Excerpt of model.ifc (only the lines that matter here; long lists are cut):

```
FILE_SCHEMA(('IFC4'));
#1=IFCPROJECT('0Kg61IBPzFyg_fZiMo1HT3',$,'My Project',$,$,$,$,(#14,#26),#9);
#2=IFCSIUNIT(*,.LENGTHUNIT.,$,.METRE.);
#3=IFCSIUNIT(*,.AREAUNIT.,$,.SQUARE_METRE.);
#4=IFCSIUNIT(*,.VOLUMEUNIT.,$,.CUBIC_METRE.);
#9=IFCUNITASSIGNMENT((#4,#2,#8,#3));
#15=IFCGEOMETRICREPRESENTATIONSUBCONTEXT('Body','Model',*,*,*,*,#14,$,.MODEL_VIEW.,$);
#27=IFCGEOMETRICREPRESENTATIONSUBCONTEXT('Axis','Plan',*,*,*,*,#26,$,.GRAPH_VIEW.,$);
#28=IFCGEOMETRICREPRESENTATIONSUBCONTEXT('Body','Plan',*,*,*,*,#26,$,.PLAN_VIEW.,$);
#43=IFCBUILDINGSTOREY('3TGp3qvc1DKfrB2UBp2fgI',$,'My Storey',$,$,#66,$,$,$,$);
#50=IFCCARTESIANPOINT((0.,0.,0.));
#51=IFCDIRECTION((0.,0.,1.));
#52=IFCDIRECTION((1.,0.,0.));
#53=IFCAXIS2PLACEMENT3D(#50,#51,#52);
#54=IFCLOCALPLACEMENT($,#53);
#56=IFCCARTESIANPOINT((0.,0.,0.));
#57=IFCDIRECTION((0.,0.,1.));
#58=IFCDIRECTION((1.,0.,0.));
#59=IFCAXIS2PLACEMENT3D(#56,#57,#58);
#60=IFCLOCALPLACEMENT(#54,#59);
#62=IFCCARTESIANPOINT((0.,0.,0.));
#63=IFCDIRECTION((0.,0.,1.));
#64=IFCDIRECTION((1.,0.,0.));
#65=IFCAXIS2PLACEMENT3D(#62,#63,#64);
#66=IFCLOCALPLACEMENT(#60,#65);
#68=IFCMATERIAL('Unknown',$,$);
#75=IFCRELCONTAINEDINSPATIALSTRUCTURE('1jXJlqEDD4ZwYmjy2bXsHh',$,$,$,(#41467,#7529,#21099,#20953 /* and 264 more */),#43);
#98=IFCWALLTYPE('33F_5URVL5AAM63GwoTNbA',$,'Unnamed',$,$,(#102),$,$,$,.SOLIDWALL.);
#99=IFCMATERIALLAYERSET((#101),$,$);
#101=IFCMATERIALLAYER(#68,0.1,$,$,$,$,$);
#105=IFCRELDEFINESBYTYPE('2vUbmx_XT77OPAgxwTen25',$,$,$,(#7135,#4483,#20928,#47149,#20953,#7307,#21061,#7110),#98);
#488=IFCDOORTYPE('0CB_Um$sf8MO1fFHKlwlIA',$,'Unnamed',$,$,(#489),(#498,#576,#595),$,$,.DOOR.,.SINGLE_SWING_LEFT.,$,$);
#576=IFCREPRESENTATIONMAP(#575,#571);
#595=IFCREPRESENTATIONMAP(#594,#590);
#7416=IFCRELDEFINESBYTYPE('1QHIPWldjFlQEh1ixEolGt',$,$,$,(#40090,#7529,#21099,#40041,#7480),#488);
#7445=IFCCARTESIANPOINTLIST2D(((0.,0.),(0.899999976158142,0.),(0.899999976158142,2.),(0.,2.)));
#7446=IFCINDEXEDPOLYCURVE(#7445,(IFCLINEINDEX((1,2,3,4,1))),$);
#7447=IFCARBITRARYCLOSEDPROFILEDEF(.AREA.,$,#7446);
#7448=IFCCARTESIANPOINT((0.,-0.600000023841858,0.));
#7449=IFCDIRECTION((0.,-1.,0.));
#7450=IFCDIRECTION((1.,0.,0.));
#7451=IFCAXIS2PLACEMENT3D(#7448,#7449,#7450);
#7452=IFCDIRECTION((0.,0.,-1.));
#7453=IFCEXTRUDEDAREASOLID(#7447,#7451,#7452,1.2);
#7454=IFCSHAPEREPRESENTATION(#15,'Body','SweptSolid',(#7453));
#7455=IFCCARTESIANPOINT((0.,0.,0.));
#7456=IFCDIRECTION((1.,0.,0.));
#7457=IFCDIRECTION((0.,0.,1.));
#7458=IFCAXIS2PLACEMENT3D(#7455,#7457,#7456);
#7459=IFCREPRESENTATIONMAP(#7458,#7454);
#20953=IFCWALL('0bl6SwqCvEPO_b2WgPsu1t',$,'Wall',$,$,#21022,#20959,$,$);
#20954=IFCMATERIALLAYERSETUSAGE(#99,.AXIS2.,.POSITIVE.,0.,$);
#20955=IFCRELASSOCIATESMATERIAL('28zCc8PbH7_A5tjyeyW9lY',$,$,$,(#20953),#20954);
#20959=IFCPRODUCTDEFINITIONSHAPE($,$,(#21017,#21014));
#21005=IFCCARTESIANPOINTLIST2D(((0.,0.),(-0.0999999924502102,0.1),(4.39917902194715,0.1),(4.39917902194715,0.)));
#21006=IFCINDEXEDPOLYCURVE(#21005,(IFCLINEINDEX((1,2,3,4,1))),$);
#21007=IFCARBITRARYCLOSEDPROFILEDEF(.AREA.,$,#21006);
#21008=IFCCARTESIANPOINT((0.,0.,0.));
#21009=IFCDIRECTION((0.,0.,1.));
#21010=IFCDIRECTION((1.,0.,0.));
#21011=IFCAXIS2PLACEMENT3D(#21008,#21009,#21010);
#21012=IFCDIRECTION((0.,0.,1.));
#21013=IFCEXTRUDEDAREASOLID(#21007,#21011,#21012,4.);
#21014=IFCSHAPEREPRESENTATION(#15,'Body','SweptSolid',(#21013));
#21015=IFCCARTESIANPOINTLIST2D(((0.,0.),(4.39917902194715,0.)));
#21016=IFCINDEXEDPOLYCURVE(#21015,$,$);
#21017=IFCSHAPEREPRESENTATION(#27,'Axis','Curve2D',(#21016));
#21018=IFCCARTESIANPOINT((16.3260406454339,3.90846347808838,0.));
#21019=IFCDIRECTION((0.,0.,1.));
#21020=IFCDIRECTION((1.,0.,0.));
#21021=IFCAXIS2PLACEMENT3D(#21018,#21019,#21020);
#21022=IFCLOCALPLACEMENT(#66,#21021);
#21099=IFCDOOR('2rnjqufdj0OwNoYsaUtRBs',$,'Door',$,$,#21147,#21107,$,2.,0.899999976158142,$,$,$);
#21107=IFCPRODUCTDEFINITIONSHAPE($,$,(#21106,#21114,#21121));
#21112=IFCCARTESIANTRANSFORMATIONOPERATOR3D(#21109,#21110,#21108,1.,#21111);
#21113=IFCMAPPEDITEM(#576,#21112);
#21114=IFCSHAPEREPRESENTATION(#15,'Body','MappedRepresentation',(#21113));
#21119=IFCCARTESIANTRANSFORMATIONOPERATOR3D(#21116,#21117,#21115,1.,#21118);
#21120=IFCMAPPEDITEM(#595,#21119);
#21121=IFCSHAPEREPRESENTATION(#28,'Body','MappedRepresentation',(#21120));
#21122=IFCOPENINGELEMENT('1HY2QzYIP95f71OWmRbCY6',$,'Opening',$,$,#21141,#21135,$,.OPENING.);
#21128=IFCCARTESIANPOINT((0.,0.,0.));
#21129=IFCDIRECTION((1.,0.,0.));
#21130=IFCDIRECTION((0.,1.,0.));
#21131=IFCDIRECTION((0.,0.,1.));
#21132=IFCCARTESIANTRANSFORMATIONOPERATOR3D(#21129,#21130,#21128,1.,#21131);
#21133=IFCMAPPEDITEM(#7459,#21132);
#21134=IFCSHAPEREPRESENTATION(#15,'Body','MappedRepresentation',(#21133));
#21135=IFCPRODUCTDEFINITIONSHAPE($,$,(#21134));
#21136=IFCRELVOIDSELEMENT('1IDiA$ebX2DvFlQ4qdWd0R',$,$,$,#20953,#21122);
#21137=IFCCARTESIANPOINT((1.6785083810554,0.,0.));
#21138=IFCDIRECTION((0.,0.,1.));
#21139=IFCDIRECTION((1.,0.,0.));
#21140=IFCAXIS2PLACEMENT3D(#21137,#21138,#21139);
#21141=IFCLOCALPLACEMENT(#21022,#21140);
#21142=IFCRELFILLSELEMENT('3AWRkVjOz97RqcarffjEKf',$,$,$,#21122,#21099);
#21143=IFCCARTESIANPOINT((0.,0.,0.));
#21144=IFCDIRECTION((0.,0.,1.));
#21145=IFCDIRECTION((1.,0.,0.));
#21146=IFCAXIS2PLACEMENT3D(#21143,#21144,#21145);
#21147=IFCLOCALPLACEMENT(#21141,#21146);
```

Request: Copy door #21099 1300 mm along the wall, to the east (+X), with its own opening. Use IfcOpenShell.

```python
import ifcopenshell
import ifcopenshell.api.feature
import ifcopenshell.api.geometry
import ifcopenshell.api.root
import ifcopenshell.geom
import ifcopenshell.util.element
import ifcopenshell.util.placement
import ifcopenshell.util.shape
import ifcopenshell.util.unit

model = ifcopenshell.open("model.ifc")
unit_scale = ifcopenshell.util.unit.calculate_unit_scale(model)
settings = ifcopenshell.geom.settings()


def volume(element):
    """Net volume in cubic metres, openings subtracted."""
    shape = ifcopenshell.geom.create_shape(settings, element)
    return ifcopenshell.util.shape.get_volume(shape.geometry)


door = model.by_id(21099)
opening = door.FillsVoids[0].RelatingOpeningElement
wall = opening.VoidsElements[0].RelatingBuildingElement
before = volume(wall)
shift = ifcopenshell.util.placement.get_local_placement(wall.ObjectPlacement)[:3, 0] * 1.3 / unit_scale

# copy_class copies the void relationship, type, container and properties, but no geometry.
new_opening = ifcopenshell.api.root.copy_class(model, product=opening)
new_opening.Representation = ifcopenshell.util.element.copy_deep(
    model, opening.Representation, exclude=["IfcGeometricRepresentationContext", "IfcRepresentationMap"]
)
new_door = ifcopenshell.api.root.copy_class(model, product=door)
new_door.Representation = ifcopenshell.util.element.copy_deep(
    model, door.Representation, exclude=["IfcGeometricRepresentationContext", "IfcRepresentationMap"]
)
ifcopenshell.api.feature.add_filling(model, opening=new_opening, element=new_door)

for old, new in ((opening, new_opening), (door, new_door)):
    matrix = ifcopenshell.util.placement.get_local_placement(old.ObjectPlacement)
    matrix[:3, 3] += shift
    ifcopenshell.api.geometry.edit_object_placement(model, product=new, matrix=matrix, is_si=False)

after = volume(wall)

print(f"wall volume {before:.3f} -> {after:.3f} m3")

model.write("model-out.ifc")
```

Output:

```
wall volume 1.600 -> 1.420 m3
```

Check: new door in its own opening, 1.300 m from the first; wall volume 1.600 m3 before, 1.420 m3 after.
